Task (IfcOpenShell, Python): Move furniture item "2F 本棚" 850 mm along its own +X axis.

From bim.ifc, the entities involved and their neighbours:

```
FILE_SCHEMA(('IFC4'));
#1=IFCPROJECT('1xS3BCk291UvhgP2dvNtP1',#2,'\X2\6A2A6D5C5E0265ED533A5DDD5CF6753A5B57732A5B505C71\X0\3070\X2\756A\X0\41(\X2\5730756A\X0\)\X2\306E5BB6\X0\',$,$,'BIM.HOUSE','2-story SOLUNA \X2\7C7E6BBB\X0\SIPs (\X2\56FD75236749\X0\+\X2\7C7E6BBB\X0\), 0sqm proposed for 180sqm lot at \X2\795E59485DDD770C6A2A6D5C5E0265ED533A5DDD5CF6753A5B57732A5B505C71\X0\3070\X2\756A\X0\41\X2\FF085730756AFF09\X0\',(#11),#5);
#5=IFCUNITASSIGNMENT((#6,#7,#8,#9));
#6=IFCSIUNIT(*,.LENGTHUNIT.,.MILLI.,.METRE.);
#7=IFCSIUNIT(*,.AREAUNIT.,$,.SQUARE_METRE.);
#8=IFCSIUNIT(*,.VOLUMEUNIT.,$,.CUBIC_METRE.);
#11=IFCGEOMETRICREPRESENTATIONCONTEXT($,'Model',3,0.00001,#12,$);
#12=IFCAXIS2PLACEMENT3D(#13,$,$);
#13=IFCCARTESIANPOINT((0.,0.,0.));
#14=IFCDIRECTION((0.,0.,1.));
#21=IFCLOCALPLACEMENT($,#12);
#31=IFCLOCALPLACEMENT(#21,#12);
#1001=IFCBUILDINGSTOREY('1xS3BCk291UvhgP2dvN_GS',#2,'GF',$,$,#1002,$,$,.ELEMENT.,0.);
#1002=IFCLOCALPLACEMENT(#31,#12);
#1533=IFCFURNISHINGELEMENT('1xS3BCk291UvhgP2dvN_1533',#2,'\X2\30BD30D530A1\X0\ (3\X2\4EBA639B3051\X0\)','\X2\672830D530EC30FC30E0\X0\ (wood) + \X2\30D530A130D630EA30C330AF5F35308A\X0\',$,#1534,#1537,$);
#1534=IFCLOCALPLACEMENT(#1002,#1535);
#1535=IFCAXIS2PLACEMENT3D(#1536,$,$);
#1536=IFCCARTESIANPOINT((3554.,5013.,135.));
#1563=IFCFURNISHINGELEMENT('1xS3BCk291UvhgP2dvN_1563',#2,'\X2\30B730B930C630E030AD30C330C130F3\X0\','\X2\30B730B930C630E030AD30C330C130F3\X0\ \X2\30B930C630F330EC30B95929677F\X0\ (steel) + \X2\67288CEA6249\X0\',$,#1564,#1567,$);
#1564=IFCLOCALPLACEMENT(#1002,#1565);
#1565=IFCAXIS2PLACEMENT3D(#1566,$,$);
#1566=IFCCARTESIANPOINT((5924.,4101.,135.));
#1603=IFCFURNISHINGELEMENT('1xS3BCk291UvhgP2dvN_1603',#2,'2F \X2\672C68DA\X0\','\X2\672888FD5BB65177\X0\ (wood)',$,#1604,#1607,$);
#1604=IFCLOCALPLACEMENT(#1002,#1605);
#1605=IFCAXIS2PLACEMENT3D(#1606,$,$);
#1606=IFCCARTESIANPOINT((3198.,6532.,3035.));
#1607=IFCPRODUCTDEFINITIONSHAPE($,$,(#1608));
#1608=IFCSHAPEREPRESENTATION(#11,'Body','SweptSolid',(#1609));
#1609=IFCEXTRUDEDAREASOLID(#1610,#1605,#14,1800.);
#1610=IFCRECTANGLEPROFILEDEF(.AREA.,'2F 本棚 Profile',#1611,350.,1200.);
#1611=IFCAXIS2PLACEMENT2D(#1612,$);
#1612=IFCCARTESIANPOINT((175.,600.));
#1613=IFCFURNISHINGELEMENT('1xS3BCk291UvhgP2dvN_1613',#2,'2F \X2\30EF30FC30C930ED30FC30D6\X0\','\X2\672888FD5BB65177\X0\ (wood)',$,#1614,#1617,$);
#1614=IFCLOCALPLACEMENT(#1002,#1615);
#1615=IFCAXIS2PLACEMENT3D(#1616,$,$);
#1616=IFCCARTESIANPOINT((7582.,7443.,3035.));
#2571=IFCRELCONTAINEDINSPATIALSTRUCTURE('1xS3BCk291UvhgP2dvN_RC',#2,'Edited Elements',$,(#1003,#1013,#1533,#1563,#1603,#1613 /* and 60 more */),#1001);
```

```python
import ifcopenshell
import ifcopenshell.api.geometry
import ifcopenshell.util.placement
import ifcopenshell.util.unit

model = ifcopenshell.open("bim.ifc")
unit_scale = ifcopenshell.util.unit.calculate_unit_scale(model)

item = model.by_guid("1xS3BCk291UvhgP2dvN_1603")
matrix = ifcopenshell.util.placement.get_local_placement(item.ObjectPlacement)
matrix[:3, 3] += matrix[:3, 0] * 0.85 / unit_scale
ifcopenshell.api.geometry.edit_object_placement(model, product=item, matrix=matrix, is_si=False)

print(ifcopenshell.util.placement.get_local_placement(item.ObjectPlacement).round(3) + 0.0)

model.write("bim_edited.ifc")
```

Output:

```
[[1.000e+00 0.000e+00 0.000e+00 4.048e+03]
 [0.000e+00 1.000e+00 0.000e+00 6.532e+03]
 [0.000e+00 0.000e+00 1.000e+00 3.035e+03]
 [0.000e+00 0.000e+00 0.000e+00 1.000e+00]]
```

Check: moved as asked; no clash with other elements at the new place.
